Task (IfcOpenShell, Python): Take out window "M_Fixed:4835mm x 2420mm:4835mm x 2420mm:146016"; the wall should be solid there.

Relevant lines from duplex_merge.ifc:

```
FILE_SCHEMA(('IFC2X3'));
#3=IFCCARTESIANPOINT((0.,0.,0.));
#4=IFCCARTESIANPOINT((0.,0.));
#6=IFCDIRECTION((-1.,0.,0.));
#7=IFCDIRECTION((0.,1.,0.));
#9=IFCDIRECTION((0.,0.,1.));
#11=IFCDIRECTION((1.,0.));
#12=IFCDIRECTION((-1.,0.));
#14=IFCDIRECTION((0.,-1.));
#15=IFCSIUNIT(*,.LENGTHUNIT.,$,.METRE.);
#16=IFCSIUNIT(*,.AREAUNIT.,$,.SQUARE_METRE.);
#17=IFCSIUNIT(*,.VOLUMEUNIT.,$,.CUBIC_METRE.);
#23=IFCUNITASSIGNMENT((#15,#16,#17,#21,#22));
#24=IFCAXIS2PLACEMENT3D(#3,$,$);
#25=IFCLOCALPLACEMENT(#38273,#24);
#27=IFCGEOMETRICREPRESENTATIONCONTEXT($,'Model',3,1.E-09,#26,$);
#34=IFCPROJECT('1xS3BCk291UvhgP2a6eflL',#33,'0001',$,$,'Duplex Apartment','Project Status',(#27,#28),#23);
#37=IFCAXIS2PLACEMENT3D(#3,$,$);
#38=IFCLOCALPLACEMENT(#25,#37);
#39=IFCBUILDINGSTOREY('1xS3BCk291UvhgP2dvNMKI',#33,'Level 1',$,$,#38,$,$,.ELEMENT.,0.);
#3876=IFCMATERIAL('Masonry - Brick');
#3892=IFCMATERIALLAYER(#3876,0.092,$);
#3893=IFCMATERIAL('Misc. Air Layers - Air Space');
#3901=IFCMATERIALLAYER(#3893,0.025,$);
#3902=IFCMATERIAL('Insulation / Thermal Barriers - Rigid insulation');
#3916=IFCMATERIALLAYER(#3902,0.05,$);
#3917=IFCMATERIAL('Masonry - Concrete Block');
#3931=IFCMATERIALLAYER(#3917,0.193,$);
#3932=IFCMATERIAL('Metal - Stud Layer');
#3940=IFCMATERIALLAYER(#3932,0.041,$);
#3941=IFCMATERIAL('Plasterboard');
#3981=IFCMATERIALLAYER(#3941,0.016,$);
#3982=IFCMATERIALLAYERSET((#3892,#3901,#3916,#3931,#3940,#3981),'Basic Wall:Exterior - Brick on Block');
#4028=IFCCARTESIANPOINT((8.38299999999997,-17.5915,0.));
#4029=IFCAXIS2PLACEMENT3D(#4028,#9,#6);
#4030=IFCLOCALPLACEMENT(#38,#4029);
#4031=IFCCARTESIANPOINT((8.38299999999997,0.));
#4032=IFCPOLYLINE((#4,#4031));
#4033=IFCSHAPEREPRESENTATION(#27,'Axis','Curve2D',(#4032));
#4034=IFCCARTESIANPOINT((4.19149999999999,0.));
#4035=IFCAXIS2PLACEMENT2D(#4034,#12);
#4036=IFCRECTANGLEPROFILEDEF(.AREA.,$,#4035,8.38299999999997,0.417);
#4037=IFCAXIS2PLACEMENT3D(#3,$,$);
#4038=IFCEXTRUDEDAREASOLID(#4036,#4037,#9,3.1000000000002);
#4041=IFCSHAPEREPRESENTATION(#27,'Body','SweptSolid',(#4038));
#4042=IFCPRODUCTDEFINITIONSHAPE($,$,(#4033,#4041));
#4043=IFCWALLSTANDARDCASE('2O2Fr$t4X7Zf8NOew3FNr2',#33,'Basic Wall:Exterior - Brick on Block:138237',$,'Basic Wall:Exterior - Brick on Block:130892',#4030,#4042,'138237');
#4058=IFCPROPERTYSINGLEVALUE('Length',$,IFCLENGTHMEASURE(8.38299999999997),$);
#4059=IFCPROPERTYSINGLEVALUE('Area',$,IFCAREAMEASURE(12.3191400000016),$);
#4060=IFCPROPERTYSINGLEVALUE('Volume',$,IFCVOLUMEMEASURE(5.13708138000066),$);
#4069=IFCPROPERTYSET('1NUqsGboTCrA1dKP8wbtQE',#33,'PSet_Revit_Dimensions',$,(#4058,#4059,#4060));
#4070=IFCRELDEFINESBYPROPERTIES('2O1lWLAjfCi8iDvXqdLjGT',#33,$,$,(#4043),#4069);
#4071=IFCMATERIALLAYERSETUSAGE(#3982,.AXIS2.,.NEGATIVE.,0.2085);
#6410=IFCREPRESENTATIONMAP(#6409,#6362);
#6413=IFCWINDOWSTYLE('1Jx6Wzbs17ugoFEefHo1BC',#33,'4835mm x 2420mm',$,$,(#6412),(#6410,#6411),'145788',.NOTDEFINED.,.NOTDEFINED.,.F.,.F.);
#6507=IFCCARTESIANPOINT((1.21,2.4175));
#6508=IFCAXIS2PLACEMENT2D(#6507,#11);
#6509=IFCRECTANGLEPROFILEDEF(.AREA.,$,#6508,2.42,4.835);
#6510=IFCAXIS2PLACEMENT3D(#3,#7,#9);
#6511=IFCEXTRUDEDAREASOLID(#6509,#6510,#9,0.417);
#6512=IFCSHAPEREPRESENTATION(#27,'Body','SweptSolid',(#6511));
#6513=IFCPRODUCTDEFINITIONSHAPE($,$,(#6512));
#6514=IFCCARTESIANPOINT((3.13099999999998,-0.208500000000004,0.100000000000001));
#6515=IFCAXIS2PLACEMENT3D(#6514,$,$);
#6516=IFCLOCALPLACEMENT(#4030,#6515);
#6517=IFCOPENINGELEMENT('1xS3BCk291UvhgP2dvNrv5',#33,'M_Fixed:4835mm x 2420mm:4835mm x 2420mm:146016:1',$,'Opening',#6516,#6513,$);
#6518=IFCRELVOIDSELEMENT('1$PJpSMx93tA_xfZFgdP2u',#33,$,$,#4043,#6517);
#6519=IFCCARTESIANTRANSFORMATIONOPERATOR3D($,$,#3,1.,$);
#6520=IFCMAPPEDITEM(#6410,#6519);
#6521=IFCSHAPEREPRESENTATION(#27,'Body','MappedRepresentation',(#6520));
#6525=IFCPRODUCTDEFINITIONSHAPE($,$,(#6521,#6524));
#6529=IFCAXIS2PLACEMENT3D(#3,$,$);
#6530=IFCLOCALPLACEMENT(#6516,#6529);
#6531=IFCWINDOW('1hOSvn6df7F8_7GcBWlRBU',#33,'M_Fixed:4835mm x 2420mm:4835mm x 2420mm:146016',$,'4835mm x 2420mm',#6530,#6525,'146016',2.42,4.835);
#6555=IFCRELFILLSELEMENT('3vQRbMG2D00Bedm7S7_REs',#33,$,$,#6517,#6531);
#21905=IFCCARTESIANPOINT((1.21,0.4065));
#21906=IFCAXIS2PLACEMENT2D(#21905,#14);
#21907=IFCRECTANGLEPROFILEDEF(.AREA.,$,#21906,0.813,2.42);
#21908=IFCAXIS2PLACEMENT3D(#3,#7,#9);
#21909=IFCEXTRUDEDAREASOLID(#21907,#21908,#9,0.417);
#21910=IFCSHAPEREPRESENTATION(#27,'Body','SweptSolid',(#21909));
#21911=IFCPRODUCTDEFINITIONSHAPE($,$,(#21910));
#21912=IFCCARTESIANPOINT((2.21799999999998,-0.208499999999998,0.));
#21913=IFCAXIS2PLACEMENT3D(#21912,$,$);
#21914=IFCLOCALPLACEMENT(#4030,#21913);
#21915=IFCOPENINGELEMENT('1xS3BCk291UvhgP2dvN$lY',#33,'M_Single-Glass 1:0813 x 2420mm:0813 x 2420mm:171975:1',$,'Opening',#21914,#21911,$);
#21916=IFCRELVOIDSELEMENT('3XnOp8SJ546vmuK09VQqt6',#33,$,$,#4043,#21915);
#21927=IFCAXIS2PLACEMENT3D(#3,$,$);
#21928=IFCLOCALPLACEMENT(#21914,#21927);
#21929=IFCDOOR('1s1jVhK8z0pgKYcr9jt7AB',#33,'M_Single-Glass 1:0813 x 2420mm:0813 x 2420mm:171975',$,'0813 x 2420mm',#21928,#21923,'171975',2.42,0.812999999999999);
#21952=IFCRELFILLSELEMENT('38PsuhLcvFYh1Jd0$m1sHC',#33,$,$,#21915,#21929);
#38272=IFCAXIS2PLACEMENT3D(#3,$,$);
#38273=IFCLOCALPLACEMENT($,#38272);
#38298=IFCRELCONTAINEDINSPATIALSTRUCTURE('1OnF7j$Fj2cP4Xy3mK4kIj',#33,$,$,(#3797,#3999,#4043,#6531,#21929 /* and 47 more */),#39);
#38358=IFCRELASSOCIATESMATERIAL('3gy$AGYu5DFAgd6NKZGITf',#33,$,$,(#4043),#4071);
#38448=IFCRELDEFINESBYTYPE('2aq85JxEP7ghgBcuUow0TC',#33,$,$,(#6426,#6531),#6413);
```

```python
import ifcopenshell
import ifcopenshell.api.feature
import ifcopenshell.api.pset
import ifcopenshell.api.root
import ifcopenshell.geom
import ifcopenshell.util.element
import ifcopenshell.util.shape
import ifcopenshell.util.unit

model = ifcopenshell.open("duplex_merge.ifc")
area_scale = ifcopenshell.util.unit.calculate_unit_scale(model, "AREAUNIT")
volume_scale = ifcopenshell.util.unit.calculate_unit_scale(model, "VOLUMEUNIT")
settings = ifcopenshell.geom.settings()


def volume(element):
    """Net volume in cubic metres, openings subtracted."""
    shape = ifcopenshell.geom.create_shape(settings, element)
    return ifcopenshell.util.shape.get_volume(shape.geometry)


window = model.by_id(6531)
opening = window.FillsVoids[0].RelatingOpeningElement
wall = opening.VoidsElements[0].RelatingBuildingElement
before = volume(wall)

ifcopenshell.api.root.remove_product(model, product=window)
ifcopenshell.api.feature.remove_feature(model, feature=opening)

after = volume(wall)
thickness = 0.417  # wall thickness in metres

# Update the wall's stored quantities.
pset = model.by_id(ifcopenshell.util.element.get_pset(wall, "PSet_Revit_Dimensions", should_inherit=False)["id"])
ifcopenshell.api.pset.edit_pset(model, pset=pset, properties={
    "Area": model.create_entity("IfcAreaMeasure", after / thickness / area_scale),
    "Volume": model.create_entity("IfcVolumeMeasure", after / volume_scale),
})

print(f"wall volume {before:.3f} -> {after:.3f} m3")

model.write("duplex_merge_v2.ifc")
```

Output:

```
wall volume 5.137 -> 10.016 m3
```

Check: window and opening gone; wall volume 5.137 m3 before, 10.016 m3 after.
